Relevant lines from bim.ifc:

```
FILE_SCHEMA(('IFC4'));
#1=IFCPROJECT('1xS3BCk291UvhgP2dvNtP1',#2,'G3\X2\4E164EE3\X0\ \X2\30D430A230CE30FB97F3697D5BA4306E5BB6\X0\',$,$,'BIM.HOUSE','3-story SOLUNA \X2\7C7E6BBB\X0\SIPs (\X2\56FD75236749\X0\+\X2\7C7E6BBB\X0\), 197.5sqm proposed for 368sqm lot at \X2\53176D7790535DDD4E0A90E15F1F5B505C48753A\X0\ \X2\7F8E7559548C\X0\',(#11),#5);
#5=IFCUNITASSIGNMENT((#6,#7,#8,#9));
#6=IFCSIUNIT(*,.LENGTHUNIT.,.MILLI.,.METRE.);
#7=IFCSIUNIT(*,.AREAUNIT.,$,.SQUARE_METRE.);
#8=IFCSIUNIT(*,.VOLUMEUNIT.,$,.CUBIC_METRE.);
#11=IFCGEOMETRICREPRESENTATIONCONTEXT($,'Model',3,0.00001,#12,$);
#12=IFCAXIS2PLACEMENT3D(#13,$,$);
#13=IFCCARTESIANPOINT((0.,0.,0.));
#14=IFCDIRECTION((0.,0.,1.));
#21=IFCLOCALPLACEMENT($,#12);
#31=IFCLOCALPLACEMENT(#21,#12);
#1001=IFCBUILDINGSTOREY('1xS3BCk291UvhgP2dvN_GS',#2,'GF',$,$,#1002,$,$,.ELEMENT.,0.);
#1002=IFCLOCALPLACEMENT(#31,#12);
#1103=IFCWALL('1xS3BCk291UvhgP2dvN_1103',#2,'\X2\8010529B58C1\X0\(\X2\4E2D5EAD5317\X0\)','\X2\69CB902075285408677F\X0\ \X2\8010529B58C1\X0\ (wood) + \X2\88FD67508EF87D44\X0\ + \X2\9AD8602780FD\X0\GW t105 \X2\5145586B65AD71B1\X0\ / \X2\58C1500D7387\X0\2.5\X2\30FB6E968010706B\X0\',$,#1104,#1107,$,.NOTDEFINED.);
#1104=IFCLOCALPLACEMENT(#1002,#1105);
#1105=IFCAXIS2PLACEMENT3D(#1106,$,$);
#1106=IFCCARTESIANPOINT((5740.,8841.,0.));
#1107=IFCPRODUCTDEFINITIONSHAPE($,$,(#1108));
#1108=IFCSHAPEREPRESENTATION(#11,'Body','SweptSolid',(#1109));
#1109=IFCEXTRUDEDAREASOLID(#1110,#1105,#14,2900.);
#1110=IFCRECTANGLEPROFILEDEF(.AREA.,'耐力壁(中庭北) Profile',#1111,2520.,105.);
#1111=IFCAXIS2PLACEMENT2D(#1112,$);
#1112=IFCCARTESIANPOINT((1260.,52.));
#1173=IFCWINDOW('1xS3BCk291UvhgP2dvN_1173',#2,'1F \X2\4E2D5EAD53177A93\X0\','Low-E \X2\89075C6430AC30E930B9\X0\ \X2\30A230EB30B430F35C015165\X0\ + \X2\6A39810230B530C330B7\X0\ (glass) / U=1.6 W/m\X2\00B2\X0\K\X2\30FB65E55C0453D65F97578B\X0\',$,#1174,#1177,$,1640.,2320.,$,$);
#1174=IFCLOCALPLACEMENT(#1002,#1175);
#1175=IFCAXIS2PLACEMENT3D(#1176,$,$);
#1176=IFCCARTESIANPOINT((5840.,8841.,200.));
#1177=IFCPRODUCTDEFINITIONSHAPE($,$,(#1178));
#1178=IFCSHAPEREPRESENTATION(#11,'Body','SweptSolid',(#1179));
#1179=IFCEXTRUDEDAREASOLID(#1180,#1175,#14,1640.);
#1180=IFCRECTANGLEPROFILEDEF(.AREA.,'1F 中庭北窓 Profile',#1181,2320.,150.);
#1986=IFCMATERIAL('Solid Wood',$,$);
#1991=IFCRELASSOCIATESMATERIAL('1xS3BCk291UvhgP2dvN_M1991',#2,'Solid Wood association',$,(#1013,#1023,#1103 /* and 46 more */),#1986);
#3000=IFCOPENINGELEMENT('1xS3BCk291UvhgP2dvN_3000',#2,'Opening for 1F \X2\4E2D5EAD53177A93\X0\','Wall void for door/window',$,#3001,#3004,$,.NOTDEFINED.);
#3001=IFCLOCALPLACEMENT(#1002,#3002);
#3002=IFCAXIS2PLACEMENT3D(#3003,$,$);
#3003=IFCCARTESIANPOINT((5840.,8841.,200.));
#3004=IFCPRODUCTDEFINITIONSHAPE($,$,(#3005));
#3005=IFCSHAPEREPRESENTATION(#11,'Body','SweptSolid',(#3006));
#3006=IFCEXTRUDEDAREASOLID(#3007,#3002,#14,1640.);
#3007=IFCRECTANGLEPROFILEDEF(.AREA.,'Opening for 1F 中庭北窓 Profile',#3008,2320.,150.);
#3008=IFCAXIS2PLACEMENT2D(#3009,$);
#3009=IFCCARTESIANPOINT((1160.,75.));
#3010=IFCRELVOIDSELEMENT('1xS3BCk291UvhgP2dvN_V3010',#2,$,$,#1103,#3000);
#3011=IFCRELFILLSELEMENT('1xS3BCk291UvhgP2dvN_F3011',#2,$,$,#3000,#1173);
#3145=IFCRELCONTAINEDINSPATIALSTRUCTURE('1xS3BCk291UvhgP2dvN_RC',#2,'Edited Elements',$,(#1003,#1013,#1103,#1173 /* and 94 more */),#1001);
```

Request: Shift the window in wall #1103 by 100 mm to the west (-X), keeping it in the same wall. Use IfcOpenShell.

```python
import ifcopenshell
import ifcopenshell.api.geometry
import ifcopenshell.util.placement

model = ifcopenshell.open("bim.ifc")

window = model.by_id(1173)
opening = window.FillsVoids[0].RelatingOpeningElement
wall = opening.VoidsElements[0].RelatingBuildingElement

wall_matrix = ifcopenshell.util.placement.get_local_placement(wall.ObjectPlacement)
shift = wall_matrix[:3, 0] * -100.0
before = ifcopenshell.util.placement.get_local_placement(window.ObjectPlacement)[:3, 3].copy()

# The window is not placed relative to its opening, so move both.
for product in (opening, window):
    matrix = ifcopenshell.util.placement.get_local_placement(product.ObjectPlacement)
    matrix[:3, 3] += shift
    ifcopenshell.api.geometry.edit_object_placement(model, product=product, matrix=matrix, is_si=False)

after = ifcopenshell.util.placement.get_local_placement(window.ObjectPlacement)[:3, 3]
print("window moved by", (after - before).round(3) + 0.0)

model.write("bim_edited.ifc")
```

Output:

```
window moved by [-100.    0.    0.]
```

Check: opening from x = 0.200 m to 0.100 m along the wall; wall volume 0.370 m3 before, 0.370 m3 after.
